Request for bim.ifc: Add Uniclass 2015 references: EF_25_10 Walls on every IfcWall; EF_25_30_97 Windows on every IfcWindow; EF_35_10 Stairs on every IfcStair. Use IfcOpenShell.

First a look at what the model holds.

```python
import ifcopenshell

model = ifcopenshell.open("bim.ifc")
print(model.schema)
print("classifications:", [c.Name for c in model.by_type("IfcClassification")])
for ifc_class in ("IfcDoor", "IfcRoof", "IfcStair", "IfcWall", "IfcWindow"):
    print(ifc_class, len(model.by_type(ifc_class)))
```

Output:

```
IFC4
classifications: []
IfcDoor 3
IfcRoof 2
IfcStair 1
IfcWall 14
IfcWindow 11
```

```python
import ifcopenshell
import ifcopenshell.api.classification

model = ifcopenshell.open("bim.ifc")

system = ifcopenshell.api.classification.add_classification(model, classification="Uniclass 2015")

codes = {
    "IfcWall": ("EF_25_10", "Walls"),
    "IfcWindow": ("EF_25_30_97", "Windows"),
    "IfcStair": ("EF_35_10", "Stairs"),
}
for ifc_class, (code, name) in codes.items():
    products = model.by_type(ifc_class)
    ifcopenshell.api.classification.add_reference(
        model, products=products, classification=system, identification=code, name=name
    )
    print(code, len(products))

model.write("bim_updated.ifc")
```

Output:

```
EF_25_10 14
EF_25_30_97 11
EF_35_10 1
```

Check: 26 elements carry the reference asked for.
